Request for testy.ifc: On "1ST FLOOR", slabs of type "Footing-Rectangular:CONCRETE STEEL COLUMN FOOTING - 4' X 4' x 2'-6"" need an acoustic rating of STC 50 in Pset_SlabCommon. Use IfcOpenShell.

First a look at what the model holds.

```python
import ifcopenshell
import ifcopenshell.util.element

model = ifcopenshell.open("testy.ifc")
print(model.schema)
storey = next(s for s in model.by_type("IfcBuildingStorey") if s.Name == "1ST FLOOR")
slabs = [e for e in ifcopenshell.util.element.get_decomposition(storey) if e.is_a("IfcSlab")]
seen = {}
for e in slabs:
    element_type = ifcopenshell.util.element.get_type(e)
    key = (element_type.Name if element_type != e and element_type else None, ifcopenshell.util.element.get_pset(e, "Pset_SlabCommon", "AcousticRating"))
    seen[key] = seen.get(key, 0) + 1
for (name, value), count in sorted(seen.items(), key=str):
    print(count, "x", name, "|", value)
```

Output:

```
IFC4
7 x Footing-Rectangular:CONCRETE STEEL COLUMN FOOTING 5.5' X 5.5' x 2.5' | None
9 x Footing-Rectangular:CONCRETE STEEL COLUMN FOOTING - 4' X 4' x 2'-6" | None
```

```python
import ifcopenshell
import ifcopenshell.api.pset
import ifcopenshell.util.element

model = ifcopenshell.open("testy.ifc")

storey = next(s for s in model.by_type("IfcBuildingStorey") if s.Name == "1ST FLOOR")
slabs = [e for e in ifcopenshell.util.element.get_decomposition(storey) if e.is_a("IfcSlab")]

count = 0
for e in slabs:
    element_type = ifcopenshell.util.element.get_type(e)
    if element_type in (None, e) or element_type.Name != 'Footing-Rectangular:CONCRETE STEEL COLUMN FOOTING - 4\' X 4\' x 2\'-6"':
        continue
    # add_pset returns the element's existing set when there is one.
    pset = ifcopenshell.api.pset.add_pset(model, product=e, name="Pset_SlabCommon")
    ifcopenshell.api.pset.edit_pset(model, pset=pset, properties={"AcousticRating": "STC 50"})
    count += 1

print(count, "slabs updated")

model.write("testy-out.ifc")
```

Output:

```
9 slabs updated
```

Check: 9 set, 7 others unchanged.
